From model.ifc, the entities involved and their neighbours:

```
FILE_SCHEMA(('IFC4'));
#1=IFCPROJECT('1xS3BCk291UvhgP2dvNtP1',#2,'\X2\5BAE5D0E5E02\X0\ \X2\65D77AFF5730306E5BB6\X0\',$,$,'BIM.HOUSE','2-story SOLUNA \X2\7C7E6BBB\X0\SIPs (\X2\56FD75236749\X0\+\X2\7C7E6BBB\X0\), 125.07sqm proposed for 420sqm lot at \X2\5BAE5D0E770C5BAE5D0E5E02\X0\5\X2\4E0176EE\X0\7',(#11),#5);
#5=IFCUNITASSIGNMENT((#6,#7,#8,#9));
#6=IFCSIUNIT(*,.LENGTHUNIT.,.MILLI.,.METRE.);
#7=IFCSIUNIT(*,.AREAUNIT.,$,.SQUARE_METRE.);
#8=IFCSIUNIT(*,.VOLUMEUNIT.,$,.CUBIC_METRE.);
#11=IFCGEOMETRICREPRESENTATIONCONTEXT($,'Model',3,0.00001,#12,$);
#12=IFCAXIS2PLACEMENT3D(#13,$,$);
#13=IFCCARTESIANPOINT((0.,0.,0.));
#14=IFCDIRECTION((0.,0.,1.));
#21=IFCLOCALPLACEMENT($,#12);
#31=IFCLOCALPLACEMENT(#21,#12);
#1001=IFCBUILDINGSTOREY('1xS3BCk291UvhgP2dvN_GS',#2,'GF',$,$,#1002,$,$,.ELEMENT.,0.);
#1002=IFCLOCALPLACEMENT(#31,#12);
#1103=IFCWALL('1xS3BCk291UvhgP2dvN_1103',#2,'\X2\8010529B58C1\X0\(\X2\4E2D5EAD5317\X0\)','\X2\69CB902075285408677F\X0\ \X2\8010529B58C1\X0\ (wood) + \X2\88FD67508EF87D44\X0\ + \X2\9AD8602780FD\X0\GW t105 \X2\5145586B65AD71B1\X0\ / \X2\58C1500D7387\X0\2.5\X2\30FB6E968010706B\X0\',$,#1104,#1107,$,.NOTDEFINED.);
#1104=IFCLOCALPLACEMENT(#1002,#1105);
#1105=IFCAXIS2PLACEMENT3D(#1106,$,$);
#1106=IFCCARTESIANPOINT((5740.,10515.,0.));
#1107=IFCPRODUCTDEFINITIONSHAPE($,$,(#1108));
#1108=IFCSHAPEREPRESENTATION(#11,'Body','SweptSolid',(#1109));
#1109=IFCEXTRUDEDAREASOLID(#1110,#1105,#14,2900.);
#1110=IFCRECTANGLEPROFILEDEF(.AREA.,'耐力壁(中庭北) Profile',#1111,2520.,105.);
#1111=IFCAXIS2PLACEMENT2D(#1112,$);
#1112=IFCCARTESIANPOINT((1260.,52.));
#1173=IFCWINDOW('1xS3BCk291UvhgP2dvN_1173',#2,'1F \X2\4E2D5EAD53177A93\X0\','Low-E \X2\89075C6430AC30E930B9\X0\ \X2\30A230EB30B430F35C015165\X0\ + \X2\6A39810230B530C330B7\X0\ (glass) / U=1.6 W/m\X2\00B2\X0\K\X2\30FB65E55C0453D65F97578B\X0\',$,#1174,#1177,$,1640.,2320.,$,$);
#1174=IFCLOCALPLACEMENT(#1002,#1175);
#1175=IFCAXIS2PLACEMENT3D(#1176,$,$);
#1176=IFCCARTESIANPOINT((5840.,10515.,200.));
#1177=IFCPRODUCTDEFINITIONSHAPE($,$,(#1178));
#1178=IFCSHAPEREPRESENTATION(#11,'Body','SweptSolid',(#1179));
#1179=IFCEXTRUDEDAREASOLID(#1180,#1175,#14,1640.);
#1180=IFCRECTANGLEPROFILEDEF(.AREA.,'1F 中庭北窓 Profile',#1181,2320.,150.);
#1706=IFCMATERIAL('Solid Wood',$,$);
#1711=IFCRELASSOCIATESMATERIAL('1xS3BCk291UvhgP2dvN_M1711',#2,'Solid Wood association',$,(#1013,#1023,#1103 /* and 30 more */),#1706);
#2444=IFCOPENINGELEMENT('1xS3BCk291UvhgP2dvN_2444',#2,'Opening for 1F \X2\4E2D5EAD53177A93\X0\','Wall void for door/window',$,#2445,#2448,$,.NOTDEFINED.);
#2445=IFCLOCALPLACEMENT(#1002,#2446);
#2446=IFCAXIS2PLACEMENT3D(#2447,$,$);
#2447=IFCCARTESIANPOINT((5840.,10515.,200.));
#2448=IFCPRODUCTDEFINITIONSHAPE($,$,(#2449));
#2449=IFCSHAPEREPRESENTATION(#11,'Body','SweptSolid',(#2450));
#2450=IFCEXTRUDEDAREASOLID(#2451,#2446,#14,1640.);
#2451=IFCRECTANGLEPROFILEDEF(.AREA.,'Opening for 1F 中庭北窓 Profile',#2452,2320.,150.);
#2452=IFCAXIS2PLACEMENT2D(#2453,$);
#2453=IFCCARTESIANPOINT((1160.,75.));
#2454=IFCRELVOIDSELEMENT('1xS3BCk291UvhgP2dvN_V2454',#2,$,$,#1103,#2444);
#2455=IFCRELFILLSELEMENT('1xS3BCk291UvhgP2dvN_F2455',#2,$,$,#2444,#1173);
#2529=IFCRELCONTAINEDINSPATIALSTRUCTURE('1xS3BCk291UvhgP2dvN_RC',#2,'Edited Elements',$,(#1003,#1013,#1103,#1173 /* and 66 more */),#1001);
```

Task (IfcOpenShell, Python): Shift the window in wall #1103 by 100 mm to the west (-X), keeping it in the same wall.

```python
import ifcopenshell
import ifcopenshell.api.geometry
import ifcopenshell.util.placement
import ifcopenshell.util.unit

model = ifcopenshell.open("model.ifc")
unit_scale = ifcopenshell.util.unit.calculate_unit_scale(model)

window = model.by_guid("1xS3BCk291UvhgP2dvN_1173")
opening = window.FillsVoids[0].RelatingOpeningElement
wall = opening.VoidsElements[0].RelatingBuildingElement

wall_matrix = ifcopenshell.util.placement.get_local_placement(wall.ObjectPlacement)
shift = wall_matrix[:3, 0] * -0.1 / unit_scale
before = ifcopenshell.util.placement.get_local_placement(window.ObjectPlacement)[:3, 3].copy()

# The window is not placed relative to its opening, so move both.
for product in (opening, window):
    matrix = ifcopenshell.util.placement.get_local_placement(product.ObjectPlacement)
    matrix[:3, 3] += shift
    ifcopenshell.api.geometry.edit_object_placement(model, product=product, matrix=matrix, is_si=False)

after = ifcopenshell.util.placement.get_local_placement(window.ObjectPlacement)[:3, 3]
print("window moved by", (after - before).round(3) + 0.0)

model.write("model_rev.ifc")
```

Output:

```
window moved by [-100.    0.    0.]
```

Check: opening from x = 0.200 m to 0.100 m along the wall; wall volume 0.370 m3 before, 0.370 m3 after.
